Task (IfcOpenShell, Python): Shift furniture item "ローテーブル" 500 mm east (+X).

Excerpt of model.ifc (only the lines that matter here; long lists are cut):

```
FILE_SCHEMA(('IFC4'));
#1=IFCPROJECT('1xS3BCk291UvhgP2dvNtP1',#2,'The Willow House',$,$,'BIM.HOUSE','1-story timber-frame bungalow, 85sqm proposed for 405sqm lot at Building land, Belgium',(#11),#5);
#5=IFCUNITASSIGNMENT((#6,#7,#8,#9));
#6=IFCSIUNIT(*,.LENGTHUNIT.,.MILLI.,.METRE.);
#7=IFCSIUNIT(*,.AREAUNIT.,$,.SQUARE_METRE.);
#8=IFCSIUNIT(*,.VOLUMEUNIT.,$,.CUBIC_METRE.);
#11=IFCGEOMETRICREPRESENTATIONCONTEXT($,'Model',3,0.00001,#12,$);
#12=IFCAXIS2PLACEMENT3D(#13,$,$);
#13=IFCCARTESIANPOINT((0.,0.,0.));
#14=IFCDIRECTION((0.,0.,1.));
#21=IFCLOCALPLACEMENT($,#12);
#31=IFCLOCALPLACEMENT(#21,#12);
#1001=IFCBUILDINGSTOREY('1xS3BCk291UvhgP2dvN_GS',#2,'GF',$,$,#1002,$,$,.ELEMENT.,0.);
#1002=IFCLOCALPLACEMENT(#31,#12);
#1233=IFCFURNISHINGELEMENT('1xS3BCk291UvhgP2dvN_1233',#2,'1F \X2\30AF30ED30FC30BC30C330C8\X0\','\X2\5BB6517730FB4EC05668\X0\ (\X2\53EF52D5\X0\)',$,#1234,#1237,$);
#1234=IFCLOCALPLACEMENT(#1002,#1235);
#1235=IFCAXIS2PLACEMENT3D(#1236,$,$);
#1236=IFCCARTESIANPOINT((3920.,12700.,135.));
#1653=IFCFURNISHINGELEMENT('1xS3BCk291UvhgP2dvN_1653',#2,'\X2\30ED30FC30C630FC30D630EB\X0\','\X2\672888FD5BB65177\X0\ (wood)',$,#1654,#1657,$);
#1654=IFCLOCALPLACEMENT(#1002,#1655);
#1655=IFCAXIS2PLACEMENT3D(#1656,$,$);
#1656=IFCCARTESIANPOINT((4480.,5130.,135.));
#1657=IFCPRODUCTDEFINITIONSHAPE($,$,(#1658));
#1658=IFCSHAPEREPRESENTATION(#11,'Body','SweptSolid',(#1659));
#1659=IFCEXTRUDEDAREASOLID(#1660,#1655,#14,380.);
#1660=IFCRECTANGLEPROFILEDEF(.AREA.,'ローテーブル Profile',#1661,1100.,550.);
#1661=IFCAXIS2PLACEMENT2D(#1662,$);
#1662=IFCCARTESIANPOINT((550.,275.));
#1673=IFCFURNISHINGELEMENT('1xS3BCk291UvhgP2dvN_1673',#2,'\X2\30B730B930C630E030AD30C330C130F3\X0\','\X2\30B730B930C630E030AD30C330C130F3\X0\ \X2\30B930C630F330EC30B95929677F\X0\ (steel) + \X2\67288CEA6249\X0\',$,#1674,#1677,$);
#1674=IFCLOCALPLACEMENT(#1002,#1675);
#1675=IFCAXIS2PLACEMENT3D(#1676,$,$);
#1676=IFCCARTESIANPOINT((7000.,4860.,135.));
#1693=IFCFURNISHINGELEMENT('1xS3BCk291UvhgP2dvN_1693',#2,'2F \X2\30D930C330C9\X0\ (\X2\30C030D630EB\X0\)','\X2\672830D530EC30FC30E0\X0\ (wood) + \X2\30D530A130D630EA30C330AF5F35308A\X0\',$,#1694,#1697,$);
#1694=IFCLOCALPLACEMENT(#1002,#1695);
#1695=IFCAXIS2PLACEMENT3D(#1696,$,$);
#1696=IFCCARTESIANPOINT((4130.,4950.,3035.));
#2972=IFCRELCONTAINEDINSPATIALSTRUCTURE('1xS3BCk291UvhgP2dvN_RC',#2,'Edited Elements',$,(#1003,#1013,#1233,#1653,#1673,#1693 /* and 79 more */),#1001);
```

```python
import ifcopenshell
import ifcopenshell.api.geometry
import ifcopenshell.util.placement

model = ifcopenshell.open("model.ifc")

item = model.by_id(1653)
matrix = ifcopenshell.util.placement.get_local_placement(item.ObjectPlacement)
matrix[0, 3] += 500.0
ifcopenshell.api.geometry.edit_object_placement(model, product=item, matrix=matrix, is_si=False)

print(ifcopenshell.util.placement.get_local_placement(item.ObjectPlacement).round(3) + 0.0)

model.write("model_edited.ifc")
```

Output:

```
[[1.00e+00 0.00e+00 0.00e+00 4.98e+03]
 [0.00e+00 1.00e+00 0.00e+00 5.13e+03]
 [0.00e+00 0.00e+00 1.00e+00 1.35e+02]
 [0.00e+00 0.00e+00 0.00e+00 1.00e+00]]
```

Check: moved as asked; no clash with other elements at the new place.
